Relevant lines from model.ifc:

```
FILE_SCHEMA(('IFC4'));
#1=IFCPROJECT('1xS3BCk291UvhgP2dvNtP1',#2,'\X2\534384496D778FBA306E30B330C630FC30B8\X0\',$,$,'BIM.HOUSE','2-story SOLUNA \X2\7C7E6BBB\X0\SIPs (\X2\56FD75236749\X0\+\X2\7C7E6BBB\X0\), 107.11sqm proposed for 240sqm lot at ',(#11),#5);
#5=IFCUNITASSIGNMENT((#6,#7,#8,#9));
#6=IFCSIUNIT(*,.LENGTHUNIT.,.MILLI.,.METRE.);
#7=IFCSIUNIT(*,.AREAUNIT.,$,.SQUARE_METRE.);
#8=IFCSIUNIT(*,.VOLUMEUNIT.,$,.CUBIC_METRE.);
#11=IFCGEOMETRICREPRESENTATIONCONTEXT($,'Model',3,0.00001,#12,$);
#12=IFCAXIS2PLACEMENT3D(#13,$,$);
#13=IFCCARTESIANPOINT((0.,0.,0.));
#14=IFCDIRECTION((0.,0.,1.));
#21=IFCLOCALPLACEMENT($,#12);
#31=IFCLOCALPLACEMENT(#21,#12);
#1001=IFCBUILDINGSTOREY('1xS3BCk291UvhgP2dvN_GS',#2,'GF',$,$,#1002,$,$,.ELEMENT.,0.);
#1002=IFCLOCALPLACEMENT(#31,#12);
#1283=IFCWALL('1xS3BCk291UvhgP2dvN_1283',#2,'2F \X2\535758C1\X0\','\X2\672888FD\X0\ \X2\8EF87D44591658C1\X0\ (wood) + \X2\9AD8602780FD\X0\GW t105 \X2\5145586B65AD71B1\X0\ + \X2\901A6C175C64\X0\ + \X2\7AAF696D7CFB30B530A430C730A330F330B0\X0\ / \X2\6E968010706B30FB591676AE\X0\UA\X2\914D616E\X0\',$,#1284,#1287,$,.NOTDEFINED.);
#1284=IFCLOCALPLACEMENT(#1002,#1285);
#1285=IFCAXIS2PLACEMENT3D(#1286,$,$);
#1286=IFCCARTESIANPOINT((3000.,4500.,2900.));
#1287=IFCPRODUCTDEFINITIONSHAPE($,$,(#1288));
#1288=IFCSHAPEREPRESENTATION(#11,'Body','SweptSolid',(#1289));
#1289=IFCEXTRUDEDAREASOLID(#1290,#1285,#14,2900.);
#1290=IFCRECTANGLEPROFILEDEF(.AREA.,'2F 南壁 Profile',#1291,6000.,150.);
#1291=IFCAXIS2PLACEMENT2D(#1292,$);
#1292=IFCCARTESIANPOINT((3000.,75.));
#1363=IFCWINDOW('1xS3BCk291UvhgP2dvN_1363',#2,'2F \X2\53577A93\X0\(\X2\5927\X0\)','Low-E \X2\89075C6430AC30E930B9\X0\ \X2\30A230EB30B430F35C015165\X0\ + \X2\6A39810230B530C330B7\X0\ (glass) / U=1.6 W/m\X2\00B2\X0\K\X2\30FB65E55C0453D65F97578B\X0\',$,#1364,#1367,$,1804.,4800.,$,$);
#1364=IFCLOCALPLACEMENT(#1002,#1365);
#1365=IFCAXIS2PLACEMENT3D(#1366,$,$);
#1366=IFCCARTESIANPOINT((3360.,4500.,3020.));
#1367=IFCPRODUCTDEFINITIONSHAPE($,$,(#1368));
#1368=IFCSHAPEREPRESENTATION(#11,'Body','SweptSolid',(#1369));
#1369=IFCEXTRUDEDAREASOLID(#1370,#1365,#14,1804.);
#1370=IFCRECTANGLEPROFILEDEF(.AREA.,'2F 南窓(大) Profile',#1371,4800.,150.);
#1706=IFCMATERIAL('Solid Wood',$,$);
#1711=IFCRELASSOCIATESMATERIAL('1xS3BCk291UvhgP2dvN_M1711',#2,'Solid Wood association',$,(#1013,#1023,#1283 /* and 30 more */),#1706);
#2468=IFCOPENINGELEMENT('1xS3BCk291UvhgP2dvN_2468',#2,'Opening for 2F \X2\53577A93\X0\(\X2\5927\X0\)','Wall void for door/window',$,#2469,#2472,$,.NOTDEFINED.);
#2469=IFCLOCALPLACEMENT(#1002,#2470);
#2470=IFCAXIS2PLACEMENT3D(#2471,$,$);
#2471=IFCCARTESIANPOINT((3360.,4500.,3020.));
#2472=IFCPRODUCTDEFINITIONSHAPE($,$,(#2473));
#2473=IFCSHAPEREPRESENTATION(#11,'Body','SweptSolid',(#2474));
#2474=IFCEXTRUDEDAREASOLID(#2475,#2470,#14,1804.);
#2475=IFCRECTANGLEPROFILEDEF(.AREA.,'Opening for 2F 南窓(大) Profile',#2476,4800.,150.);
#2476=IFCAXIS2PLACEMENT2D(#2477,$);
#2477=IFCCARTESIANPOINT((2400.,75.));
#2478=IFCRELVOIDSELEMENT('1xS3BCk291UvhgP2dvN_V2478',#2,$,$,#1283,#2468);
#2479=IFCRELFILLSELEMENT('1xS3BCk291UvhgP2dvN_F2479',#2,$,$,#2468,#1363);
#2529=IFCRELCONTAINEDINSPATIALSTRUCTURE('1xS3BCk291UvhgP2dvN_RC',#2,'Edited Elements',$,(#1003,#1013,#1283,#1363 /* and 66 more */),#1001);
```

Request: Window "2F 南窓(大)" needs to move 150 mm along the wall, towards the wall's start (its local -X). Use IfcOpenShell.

```python
import ifcopenshell
import ifcopenshell.api.geometry
import ifcopenshell.util.placement

model = ifcopenshell.open("model.ifc")

window = model.by_guid("1xS3BCk291UvhgP2dvN_1363")
opening = window.FillsVoids[0].RelatingOpeningElement
wall = opening.VoidsElements[0].RelatingBuildingElement

wall_matrix = ifcopenshell.util.placement.get_local_placement(wall.ObjectPlacement)
shift = wall_matrix[:3, 0] * -150.0
before = ifcopenshell.util.placement.get_local_placement(window.ObjectPlacement)[:3, 3].copy()

# The window is not placed relative to its opening, so move both.
for product in (opening, window):
    matrix = ifcopenshell.util.placement.get_local_placement(product.ObjectPlacement)
    matrix[:3, 3] += shift
    ifcopenshell.api.geometry.edit_object_placement(model, product=product, matrix=matrix, is_si=False)

after = ifcopenshell.util.placement.get_local_placement(window.ObjectPlacement)[:3, 3]
print("window moved by", (after - before).round(3) + 0.0)

model.write("model_v2.ifc")
```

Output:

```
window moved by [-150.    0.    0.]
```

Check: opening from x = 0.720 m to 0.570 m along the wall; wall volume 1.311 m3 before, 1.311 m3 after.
